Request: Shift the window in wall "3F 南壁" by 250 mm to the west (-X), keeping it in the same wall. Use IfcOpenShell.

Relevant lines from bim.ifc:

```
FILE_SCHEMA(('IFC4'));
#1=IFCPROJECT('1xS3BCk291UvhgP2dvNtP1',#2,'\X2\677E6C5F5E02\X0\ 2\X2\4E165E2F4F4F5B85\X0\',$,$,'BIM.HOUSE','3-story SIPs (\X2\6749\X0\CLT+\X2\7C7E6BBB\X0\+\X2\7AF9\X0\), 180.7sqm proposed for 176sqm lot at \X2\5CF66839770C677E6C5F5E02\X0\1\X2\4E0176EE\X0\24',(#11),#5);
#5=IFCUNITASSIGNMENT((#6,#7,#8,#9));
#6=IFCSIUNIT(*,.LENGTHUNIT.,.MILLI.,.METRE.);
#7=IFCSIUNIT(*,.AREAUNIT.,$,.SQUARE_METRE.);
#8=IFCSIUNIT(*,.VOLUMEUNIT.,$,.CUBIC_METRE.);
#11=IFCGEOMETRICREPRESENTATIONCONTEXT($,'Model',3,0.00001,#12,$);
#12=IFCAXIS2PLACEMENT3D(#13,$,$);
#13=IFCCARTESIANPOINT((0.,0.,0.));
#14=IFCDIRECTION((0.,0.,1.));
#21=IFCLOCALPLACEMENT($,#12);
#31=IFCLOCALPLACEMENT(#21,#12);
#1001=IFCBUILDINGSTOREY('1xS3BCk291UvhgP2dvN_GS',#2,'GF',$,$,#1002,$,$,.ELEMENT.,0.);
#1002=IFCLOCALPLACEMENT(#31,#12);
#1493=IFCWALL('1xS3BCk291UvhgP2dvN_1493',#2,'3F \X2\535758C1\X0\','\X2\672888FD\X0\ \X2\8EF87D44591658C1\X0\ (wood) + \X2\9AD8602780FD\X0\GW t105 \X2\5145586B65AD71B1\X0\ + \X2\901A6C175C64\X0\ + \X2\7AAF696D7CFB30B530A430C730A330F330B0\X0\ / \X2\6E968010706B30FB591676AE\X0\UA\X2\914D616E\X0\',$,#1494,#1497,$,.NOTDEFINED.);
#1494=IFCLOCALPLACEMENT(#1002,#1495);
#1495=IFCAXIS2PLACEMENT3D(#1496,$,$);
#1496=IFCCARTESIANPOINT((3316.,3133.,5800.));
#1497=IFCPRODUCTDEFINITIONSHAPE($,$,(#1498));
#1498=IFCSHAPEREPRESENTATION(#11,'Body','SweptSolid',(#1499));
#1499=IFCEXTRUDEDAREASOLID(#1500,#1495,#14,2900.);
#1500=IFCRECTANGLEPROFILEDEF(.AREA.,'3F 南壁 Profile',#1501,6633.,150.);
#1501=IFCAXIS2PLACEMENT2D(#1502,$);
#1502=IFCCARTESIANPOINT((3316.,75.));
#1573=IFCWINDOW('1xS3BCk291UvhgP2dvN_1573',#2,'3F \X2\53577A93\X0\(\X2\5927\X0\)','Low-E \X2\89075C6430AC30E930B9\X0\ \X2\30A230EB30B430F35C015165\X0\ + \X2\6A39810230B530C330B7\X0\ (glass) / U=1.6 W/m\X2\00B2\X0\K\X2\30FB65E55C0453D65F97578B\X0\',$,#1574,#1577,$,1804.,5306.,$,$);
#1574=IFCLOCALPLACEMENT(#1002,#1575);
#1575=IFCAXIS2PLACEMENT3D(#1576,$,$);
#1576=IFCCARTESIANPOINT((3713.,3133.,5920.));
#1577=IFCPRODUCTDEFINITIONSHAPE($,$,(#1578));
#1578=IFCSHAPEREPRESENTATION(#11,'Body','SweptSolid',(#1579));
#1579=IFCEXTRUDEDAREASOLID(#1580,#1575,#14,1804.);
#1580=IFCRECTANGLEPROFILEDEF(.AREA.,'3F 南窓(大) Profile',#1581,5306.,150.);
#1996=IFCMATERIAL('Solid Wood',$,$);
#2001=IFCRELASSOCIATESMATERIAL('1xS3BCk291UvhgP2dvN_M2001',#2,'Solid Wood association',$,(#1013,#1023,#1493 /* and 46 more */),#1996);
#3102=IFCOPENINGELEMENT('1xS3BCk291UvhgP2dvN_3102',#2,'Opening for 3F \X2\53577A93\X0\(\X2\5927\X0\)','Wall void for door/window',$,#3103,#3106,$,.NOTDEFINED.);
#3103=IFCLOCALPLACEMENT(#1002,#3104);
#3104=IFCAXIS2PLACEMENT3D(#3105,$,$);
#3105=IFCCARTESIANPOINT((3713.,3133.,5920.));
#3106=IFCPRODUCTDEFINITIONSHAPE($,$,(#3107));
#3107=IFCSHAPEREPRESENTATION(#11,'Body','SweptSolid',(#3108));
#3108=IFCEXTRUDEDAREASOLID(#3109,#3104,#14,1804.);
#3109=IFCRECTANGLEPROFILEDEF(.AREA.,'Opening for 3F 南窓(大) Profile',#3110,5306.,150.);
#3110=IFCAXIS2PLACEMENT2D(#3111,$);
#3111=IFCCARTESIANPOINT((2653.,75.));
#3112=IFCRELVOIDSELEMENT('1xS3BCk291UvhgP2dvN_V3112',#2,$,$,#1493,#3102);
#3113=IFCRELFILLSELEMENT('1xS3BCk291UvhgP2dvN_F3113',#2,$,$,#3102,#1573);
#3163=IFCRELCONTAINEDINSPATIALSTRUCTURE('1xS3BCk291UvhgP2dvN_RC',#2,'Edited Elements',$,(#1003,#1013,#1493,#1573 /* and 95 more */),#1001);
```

```python
import ifcopenshell
import ifcopenshell.api.geometry
import ifcopenshell.util.placement
import ifcopenshell.util.unit

model = ifcopenshell.open("bim.ifc")
unit_scale = ifcopenshell.util.unit.calculate_unit_scale(model)

window = model.by_guid("1xS3BCk291UvhgP2dvN_1573")
opening = window.FillsVoids[0].RelatingOpeningElement
wall = opening.VoidsElements[0].RelatingBuildingElement

wall_matrix = ifcopenshell.util.placement.get_local_placement(wall.ObjectPlacement)
shift = wall_matrix[:3, 0] * -0.25 / unit_scale
before = ifcopenshell.util.placement.get_local_placement(window.ObjectPlacement)[:3, 3].copy()

# The window is not placed relative to its opening, so move both.
for product in (opening, window):
    matrix = ifcopenshell.util.placement.get_local_placement(product.ObjectPlacement)
    matrix[:3, 3] += shift
    ifcopenshell.api.geometry.edit_object_placement(model, product=product, matrix=matrix, is_si=False)

after = ifcopenshell.util.placement.get_local_placement(window.ObjectPlacement)[:3, 3]
print("window moved by", (after - before).round(3) + 0.0)

model.write("bim-out.ifc")
```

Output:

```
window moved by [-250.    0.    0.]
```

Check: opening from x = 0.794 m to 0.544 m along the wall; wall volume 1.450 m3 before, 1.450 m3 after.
